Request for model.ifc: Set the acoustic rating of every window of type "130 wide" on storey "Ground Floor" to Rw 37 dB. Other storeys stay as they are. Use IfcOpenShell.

First a look at what the model holds.

```python
import ifcopenshell
import ifcopenshell.util.element

model = ifcopenshell.open("model.ifc")
print(model.schema)
storey = next(s for s in model.by_type("IfcBuildingStorey") if s.Name == "Ground Floor")
windows = [e for e in ifcopenshell.util.element.get_decomposition(storey) if e.is_a("IfcWindow")]
seen = {}
for e in windows:
    element_type = ifcopenshell.util.element.get_type(e)
    key = (element_type.Name if element_type != e and element_type else None, ifcopenshell.util.element.get_pset(e, "Pset_WindowCommon", "AcousticRating"))
    seen[key] = seen.get(key, 0) + 1
for (name, value), count in sorted(seen.items(), key=str):
    print(count, "x", name, "|", value)
```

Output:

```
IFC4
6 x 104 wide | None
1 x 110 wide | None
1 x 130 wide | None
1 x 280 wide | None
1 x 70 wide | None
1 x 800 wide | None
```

```python
import ifcopenshell
import ifcopenshell.api.pset
import ifcopenshell.util.element

model = ifcopenshell.open("model.ifc")

storey = next(s for s in model.by_type("IfcBuildingStorey") if s.Name == "Ground Floor")
windows = [e for e in ifcopenshell.util.element.get_decomposition(storey) if e.is_a("IfcWindow")]

count = 0
for e in windows:
    element_type = ifcopenshell.util.element.get_type(e)
    if element_type in (None, e) or element_type.Name != "130 wide":
        continue
    # add_pset returns the element's existing set when there is one.
    pset = ifcopenshell.api.pset.add_pset(model, product=e, name="Pset_WindowCommon")
    ifcopenshell.api.pset.edit_pset(model, pset=pset, properties={"AcousticRating": "Rw 37 dB"})
    count += 1

print(count, "windows updated")

model.write("model_edited.ifc")
```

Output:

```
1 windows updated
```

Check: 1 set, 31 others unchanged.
